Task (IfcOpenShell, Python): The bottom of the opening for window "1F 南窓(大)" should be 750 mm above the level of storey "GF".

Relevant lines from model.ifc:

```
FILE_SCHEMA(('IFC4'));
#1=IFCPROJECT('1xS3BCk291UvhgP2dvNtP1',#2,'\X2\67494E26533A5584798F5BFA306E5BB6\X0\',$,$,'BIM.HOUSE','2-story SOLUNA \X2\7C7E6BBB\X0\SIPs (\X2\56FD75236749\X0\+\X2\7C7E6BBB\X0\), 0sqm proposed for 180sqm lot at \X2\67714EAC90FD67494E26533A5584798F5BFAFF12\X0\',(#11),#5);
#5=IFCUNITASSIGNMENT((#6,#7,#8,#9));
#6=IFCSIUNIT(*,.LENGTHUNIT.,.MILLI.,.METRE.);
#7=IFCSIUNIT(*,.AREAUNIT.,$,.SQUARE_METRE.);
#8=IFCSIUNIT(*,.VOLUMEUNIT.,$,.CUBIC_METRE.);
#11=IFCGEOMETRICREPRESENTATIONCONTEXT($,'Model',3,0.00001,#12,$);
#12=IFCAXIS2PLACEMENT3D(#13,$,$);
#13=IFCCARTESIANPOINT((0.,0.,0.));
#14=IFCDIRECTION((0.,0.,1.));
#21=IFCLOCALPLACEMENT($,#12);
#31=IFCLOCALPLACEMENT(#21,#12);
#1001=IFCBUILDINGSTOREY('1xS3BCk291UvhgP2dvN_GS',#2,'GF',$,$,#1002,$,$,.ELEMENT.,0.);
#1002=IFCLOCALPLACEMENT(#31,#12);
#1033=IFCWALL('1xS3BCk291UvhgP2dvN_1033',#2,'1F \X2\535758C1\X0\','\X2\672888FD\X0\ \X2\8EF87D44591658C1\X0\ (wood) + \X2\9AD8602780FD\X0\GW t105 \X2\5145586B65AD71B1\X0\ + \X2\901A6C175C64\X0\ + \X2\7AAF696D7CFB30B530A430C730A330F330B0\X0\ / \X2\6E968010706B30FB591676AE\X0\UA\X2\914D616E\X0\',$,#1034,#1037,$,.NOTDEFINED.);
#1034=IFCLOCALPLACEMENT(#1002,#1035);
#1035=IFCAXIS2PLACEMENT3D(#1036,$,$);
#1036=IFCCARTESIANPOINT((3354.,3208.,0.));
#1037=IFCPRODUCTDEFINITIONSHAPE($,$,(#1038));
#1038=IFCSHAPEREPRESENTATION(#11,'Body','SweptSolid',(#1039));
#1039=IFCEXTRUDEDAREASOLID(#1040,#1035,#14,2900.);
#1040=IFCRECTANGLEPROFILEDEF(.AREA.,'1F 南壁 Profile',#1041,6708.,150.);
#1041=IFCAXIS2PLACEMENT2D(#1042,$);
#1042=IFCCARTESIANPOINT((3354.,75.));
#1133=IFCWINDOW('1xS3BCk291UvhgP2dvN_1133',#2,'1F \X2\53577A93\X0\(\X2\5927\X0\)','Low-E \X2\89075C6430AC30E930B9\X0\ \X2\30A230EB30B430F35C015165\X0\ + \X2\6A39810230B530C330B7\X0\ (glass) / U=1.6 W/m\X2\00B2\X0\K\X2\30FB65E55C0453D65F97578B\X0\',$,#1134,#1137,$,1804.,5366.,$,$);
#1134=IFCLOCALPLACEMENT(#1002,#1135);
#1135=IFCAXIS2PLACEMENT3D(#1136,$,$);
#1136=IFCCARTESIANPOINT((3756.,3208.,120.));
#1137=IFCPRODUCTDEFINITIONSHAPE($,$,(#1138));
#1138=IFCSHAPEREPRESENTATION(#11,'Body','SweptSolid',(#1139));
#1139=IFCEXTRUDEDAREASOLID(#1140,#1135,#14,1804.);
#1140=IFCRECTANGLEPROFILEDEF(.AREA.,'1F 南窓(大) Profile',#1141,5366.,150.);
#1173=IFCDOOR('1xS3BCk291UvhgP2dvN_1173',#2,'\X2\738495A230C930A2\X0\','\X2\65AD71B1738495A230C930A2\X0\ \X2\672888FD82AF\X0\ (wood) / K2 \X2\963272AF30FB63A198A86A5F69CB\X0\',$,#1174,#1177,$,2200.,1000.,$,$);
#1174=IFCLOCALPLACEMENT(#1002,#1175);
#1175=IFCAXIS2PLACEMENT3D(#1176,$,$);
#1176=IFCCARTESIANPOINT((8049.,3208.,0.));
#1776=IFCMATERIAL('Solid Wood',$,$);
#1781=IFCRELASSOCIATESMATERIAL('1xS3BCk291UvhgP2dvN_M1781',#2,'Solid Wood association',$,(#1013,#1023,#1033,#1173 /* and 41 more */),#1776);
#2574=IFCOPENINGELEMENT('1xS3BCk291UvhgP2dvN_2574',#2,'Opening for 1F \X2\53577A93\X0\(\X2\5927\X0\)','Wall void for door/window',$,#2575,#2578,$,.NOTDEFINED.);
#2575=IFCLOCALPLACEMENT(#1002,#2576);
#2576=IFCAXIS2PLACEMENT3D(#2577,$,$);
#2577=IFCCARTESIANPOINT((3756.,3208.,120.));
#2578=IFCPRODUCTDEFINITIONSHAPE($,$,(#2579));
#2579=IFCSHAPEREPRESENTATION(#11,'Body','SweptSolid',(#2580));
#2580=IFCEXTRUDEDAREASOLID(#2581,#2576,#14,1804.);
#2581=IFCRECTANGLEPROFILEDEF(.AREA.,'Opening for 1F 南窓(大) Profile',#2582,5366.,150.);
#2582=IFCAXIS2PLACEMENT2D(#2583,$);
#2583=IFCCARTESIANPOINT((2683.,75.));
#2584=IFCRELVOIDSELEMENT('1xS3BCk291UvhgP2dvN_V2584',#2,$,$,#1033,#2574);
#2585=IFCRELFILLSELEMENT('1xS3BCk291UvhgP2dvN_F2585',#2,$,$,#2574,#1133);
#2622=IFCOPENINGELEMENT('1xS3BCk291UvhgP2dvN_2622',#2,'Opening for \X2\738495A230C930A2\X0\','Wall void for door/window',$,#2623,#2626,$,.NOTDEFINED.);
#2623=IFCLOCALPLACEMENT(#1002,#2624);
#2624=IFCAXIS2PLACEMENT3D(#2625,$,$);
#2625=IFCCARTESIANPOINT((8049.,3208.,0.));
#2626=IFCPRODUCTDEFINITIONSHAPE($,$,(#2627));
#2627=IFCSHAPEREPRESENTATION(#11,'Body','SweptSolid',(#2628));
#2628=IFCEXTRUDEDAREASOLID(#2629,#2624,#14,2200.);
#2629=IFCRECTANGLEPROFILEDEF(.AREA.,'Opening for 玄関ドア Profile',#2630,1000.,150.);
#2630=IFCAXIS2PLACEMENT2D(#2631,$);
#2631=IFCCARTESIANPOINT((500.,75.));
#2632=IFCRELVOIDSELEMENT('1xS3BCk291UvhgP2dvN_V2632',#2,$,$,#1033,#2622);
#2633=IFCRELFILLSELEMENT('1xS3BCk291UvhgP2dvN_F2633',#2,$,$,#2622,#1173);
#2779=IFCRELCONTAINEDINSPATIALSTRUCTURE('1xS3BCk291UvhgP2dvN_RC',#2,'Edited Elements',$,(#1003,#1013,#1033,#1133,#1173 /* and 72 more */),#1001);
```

```python
import numpy as np
import ifcopenshell
import ifcopenshell.api.geometry
import ifcopenshell.geom
import ifcopenshell.util.element
import ifcopenshell.util.placement
import ifcopenshell.util.shape
import ifcopenshell.util.unit

model = ifcopenshell.open("model.ifc")
unit_scale = ifcopenshell.util.unit.calculate_unit_scale(model)

window = model.by_guid("1xS3BCk291UvhgP2dvN_1133")
opening = window.FillsVoids[0].RelatingOpeningElement
storey = ifcopenshell.util.element.get_container(window, ifc_class="IfcBuildingStorey")
level = ifcopenshell.util.placement.get_local_placement(storey.ObjectPlacement)[2, 3]

# The opening's origin need not be at the sill, so measure its lowest point.
shape = ifcopenshell.geom.create_shape(ifcopenshell.geom.settings(), opening)
bottom = ifcopenshell.util.shape.get_shape_bottom_elevation(shape, shape.geometry) / unit_scale
dz = level + 750.0 - bottom

shift = np.array([0.0, 0.0, dz])
# The window is not placed relative to its opening, so move both.
for product in (opening, window):
    matrix = ifcopenshell.util.placement.get_local_placement(product.ObjectPlacement)
    matrix[:3, 3] += shift
    ifcopenshell.api.geometry.edit_object_placement(model, product=product, matrix=matrix, is_si=False)

print(f"moved by {dz * unit_scale:+.3f} m")

model.write("model_updated.ifc")
```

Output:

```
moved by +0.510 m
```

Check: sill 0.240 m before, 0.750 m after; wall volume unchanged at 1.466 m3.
